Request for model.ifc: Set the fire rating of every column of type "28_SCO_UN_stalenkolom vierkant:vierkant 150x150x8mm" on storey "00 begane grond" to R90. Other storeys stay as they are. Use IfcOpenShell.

First a look at what the model holds.

```python
import ifcopenshell
import ifcopenshell.util.element

model = ifcopenshell.open("model.ifc")
print(model.schema)
storey = next(s for s in model.by_type("IfcBuildingStorey") if s.Name == "00 begane grond")
columns = [e for e in ifcopenshell.util.element.get_decomposition(storey) if e.is_a("IfcColumn")]
seen = {}
for e in columns:
    element_type = ifcopenshell.util.element.get_type(e)
    key = (element_type.Name if element_type != e and element_type else None, ifcopenshell.util.element.get_pset(e, "Pset_ColumnCommon", "FireRating"))
    seen[key] = seen.get(key, 0) + 1
for (name, value), count in sorted(seen.items(), key=str):
    print(count, "x", name, "|", value)
```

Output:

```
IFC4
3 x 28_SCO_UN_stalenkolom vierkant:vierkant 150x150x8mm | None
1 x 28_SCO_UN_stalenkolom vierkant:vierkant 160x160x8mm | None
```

```python
import ifcopenshell
import ifcopenshell.api.pset
import ifcopenshell.util.element

model = ifcopenshell.open("model.ifc")

storey = next(s for s in model.by_type("IfcBuildingStorey") if s.Name == "00 begane grond")
columns = [e for e in ifcopenshell.util.element.get_decomposition(storey) if e.is_a("IfcColumn")]

count = 0
for e in columns:
    element_type = ifcopenshell.util.element.get_type(e)
    if element_type in (None, e) or element_type.Name != "28_SCO_UN_stalenkolom vierkant:vierkant 150x150x8mm":
        continue
    # add_pset returns the element's existing set when there is one.
    pset = ifcopenshell.api.pset.add_pset(model, product=e, name="Pset_ColumnCommon")
    ifcopenshell.api.pset.edit_pset(model, pset=pset, properties={"FireRating": "R90"})
    count += 1

print(count, "columns updated")

model.write("model_edited.ifc")
```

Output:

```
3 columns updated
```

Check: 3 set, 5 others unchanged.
